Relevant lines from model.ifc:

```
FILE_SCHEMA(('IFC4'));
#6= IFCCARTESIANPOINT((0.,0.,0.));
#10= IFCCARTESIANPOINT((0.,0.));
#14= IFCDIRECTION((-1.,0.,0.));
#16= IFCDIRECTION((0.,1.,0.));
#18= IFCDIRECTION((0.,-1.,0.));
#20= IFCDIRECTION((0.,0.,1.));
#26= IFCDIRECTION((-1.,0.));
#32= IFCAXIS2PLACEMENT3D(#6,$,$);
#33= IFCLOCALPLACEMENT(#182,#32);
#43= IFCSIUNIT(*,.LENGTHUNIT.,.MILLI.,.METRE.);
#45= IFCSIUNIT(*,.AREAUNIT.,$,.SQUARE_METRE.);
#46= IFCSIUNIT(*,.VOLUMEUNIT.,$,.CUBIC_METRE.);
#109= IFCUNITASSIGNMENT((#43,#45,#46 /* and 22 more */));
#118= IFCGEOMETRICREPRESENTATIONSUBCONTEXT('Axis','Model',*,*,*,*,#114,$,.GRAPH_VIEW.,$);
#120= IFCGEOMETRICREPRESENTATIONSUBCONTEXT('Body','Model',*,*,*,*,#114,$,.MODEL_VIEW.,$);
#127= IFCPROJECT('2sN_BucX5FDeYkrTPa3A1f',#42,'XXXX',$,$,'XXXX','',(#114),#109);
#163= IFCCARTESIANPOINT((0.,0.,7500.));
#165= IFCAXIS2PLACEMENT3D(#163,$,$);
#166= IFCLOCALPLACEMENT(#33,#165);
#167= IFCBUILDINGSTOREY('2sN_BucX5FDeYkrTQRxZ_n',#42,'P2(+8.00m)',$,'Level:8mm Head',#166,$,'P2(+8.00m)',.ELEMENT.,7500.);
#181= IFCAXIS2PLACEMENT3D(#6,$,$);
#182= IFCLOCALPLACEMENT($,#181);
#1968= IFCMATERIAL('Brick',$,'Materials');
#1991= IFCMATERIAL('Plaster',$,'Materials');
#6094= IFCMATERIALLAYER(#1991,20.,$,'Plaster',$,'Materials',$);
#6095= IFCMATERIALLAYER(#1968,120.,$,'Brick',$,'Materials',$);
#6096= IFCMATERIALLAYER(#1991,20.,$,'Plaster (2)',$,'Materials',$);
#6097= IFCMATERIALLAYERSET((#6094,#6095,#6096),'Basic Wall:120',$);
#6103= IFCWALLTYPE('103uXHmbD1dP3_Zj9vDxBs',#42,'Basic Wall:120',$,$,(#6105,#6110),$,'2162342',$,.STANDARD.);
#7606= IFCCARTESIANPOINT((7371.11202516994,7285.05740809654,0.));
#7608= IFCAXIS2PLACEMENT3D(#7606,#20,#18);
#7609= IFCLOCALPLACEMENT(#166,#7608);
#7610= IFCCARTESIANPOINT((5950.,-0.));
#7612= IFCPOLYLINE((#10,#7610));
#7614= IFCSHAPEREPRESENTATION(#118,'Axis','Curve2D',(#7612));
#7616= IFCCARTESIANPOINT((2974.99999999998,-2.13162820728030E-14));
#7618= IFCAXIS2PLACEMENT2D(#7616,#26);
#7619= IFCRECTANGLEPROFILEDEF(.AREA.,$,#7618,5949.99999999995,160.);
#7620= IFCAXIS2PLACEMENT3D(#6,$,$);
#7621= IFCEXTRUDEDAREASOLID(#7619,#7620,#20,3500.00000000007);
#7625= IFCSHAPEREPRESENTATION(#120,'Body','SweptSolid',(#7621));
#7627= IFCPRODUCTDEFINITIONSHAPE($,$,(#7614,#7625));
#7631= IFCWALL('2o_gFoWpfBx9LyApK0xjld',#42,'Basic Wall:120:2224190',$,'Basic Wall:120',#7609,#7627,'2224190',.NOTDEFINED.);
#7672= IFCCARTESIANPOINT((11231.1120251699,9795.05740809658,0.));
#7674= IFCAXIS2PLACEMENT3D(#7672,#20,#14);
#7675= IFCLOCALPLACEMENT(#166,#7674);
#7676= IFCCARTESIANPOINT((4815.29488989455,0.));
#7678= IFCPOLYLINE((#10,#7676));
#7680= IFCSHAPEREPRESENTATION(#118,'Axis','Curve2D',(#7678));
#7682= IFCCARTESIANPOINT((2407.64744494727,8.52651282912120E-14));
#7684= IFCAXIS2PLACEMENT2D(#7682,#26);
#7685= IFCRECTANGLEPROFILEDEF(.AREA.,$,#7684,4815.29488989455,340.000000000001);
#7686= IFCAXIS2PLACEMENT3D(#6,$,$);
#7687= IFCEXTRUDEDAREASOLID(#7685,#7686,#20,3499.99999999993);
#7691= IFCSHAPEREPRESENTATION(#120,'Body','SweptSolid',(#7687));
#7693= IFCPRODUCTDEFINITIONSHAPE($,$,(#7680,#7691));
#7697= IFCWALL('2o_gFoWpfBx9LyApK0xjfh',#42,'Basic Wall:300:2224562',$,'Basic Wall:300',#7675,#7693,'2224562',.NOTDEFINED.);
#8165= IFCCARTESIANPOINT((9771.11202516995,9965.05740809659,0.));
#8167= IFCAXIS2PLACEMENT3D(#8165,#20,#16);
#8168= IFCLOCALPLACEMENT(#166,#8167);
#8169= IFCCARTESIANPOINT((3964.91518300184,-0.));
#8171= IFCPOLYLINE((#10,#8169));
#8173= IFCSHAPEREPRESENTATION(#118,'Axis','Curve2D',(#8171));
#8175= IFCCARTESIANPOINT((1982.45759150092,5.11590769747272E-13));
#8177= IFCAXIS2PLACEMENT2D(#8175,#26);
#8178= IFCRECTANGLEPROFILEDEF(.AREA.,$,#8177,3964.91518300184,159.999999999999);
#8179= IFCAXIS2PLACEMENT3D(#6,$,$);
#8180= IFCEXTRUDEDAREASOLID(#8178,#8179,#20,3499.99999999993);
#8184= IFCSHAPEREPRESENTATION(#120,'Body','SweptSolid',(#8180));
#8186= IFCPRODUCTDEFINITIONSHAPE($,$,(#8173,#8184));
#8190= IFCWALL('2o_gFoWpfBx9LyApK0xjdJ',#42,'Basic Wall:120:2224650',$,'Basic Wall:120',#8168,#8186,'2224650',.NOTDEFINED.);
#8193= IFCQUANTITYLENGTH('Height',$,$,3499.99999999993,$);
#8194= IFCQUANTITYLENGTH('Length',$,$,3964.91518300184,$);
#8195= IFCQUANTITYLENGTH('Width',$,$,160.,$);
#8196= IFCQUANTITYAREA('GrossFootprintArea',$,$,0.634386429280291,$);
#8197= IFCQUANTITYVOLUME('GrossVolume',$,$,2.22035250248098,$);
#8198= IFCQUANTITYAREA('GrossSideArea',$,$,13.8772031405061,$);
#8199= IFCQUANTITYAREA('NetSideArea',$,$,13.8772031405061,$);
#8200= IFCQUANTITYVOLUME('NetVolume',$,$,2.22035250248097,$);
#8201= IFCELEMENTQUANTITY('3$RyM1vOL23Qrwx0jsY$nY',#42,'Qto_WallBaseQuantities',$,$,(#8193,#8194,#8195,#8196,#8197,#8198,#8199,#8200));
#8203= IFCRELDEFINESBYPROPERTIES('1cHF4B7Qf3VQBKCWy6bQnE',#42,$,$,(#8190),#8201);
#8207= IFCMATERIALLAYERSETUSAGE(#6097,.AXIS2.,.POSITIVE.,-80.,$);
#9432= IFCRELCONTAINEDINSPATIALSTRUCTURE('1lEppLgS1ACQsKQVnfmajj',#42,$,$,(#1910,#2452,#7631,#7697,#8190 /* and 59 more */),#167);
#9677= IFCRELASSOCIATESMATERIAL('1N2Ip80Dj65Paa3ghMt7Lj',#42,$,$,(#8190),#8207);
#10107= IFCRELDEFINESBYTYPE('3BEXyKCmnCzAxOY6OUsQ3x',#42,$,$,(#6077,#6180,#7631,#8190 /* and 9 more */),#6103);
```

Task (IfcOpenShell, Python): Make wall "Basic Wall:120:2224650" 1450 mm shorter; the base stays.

```python
import ifcopenshell
import ifcopenshell.api.pset
import ifcopenshell.geom
import ifcopenshell.util.element
import ifcopenshell.util.representation
import ifcopenshell.util.shape
import ifcopenshell.util.unit

model = ifcopenshell.open("model.ifc")
unit_scale = ifcopenshell.util.unit.calculate_unit_scale(model)
area_scale = ifcopenshell.util.unit.calculate_unit_scale(model, "AREAUNIT")
volume_scale = ifcopenshell.util.unit.calculate_unit_scale(model, "VOLUMEUNIT")
settings = ifcopenshell.geom.settings()


def volume(element):
    """Net volume in cubic metres, openings subtracted."""
    shape = ifcopenshell.geom.create_shape(settings, element)
    return ifcopenshell.util.shape.get_volume(shape.geometry)


wall = model.by_id(8190)
before = volume(wall)

body = ifcopenshell.util.representation.get_representation(wall, "Model", "Body")
solid = body.Items[0]
old_height = solid.Depth
solid.Depth -= 1450.0
after = volume(wall)
thickness = 0.16  # wall thickness in metres

# Update the stored height, areas and volumes.
qto = model.by_id(ifcopenshell.util.element.get_pset(wall, "Qto_WallBaseQuantities", should_inherit=False)["id"])
ifcopenshell.api.pset.edit_qto(model, qto=qto, properties={
    "Height": solid.Depth,
    "GrossVolume": ifcopenshell.util.element.get_pset(wall, "Qto_WallBaseQuantities", "GrossVolume") * solid.Depth / old_height,
    "GrossSideArea": ifcopenshell.util.element.get_pset(wall, "Qto_WallBaseQuantities", "GrossSideArea") * solid.Depth / old_height,
    "NetSideArea": after / thickness / area_scale,
    "NetVolume": after / volume_scale,
})

print(f"height {old_height:g} -> {solid.Depth:g}, volume {before:.3f} -> {after:.3f} m3")

model.write("model-out.ifc")
```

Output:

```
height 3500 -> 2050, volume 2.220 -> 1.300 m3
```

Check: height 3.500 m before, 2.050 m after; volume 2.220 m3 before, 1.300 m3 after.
